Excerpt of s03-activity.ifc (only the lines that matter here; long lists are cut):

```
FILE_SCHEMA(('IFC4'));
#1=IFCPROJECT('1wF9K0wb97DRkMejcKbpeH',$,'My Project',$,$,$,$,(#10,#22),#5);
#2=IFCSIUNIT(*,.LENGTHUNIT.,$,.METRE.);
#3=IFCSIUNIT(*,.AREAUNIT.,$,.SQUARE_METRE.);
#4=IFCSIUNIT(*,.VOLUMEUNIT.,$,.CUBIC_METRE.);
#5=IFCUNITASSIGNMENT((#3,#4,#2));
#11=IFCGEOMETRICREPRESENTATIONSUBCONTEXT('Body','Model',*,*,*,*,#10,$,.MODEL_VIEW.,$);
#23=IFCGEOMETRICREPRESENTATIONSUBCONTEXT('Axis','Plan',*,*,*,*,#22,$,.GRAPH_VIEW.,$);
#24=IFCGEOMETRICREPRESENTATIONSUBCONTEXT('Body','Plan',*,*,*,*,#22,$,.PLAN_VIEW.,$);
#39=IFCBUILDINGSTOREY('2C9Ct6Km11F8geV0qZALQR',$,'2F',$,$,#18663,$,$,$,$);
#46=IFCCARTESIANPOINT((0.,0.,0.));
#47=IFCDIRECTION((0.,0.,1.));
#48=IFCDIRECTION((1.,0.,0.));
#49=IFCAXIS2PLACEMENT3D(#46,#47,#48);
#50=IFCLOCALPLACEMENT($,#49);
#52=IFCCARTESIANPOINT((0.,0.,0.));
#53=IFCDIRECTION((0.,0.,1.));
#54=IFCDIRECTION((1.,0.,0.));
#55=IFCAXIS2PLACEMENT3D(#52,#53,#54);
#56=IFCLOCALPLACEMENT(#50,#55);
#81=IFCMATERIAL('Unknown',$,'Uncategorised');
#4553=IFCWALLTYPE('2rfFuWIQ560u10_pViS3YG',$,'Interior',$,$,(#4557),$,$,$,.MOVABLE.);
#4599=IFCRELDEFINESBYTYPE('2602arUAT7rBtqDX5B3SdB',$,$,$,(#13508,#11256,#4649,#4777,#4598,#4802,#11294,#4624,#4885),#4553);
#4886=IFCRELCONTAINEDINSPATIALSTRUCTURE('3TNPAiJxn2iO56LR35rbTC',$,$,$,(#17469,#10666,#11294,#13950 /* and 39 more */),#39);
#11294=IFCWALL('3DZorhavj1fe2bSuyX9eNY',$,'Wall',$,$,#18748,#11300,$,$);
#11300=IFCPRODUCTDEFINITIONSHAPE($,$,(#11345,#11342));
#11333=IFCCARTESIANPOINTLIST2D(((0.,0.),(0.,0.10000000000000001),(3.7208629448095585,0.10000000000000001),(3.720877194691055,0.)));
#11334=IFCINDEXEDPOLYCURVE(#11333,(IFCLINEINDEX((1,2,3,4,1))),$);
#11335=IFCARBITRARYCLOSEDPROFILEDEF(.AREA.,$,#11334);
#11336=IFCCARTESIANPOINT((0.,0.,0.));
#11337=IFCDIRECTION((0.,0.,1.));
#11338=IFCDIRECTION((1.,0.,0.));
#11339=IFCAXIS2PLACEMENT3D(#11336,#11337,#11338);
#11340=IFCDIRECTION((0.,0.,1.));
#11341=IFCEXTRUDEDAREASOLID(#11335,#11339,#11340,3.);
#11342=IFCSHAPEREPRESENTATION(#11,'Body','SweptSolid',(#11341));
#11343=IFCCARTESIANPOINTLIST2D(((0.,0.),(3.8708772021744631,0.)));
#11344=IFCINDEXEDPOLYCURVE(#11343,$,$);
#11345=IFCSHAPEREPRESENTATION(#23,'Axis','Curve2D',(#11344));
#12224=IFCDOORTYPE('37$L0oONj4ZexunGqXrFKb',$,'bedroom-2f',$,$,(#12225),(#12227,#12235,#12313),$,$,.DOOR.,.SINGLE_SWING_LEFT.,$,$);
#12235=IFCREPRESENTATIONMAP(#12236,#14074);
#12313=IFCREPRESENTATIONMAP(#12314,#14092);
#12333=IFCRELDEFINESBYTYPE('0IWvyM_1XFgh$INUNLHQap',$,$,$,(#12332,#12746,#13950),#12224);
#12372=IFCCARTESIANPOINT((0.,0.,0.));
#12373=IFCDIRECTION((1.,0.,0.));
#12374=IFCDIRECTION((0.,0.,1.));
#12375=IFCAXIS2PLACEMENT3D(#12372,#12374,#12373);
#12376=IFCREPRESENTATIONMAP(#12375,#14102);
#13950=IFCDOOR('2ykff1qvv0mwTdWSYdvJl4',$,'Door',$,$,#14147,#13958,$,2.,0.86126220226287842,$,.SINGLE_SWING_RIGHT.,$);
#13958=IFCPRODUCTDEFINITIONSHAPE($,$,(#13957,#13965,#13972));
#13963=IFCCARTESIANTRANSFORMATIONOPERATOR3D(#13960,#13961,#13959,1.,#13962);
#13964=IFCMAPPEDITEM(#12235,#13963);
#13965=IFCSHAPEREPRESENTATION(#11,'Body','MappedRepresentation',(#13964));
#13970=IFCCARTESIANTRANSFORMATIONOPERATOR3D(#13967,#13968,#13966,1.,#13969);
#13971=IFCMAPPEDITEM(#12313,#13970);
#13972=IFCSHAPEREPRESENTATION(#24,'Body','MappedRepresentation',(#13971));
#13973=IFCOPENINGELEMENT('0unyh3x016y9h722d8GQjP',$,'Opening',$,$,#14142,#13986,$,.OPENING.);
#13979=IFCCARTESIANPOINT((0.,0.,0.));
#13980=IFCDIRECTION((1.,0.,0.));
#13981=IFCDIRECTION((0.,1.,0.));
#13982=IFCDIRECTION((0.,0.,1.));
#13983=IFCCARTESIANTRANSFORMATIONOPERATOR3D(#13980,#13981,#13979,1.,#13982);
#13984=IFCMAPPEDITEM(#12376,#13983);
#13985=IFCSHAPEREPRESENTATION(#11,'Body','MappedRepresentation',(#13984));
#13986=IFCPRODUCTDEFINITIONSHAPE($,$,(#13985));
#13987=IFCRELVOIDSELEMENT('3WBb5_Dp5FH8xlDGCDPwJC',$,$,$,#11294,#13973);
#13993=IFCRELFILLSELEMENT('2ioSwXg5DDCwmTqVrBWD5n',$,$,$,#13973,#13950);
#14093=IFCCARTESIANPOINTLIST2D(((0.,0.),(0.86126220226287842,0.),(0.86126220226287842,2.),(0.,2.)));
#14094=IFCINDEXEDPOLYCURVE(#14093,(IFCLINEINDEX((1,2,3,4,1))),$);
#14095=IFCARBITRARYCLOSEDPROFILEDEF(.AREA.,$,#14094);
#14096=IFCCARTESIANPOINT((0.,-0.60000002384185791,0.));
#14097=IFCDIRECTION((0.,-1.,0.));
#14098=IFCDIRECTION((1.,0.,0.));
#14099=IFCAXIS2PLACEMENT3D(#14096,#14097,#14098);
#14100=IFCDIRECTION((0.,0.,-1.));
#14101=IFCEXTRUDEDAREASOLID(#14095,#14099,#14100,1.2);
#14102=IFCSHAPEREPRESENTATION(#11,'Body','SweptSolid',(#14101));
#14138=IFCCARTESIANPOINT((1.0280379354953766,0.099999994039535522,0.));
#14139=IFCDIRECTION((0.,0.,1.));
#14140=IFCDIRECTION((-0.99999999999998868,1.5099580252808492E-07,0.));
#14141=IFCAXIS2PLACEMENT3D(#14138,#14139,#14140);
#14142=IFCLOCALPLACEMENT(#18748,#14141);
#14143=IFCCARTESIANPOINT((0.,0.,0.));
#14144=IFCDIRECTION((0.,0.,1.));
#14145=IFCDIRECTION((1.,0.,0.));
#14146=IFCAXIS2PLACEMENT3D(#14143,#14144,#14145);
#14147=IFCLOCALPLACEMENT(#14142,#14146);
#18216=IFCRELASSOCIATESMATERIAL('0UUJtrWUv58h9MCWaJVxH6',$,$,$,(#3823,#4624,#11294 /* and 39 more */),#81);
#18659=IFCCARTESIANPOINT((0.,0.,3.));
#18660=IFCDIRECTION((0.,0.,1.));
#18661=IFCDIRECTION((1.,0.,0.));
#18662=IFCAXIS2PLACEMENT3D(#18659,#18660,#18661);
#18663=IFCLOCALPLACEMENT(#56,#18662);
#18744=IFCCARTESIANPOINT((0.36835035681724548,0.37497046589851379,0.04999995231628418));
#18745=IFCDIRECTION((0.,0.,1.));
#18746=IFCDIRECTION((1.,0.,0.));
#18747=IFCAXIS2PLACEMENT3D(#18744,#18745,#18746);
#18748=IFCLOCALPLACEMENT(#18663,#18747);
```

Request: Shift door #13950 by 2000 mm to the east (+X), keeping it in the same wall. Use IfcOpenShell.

```python
import ifcopenshell
import ifcopenshell.api.geometry
import ifcopenshell.util.placement
import ifcopenshell.util.unit

model = ifcopenshell.open("s03-activity.ifc")
unit_scale = ifcopenshell.util.unit.calculate_unit_scale(model)

door = model.by_id(13950)
opening = door.FillsVoids[0].RelatingOpeningElement
wall = opening.VoidsElements[0].RelatingBuildingElement

wall_matrix = ifcopenshell.util.placement.get_local_placement(wall.ObjectPlacement)
shift = wall_matrix[:3, 0] * 2 / unit_scale
before = ifcopenshell.util.placement.get_local_placement(door.ObjectPlacement)[:3, 3].copy()

# The door is placed relative to its opening, so it follows when the opening moves.
matrix = ifcopenshell.util.placement.get_local_placement(opening.ObjectPlacement)
matrix[:3, 3] += shift
ifcopenshell.api.geometry.edit_object_placement(
    model, product=opening, matrix=matrix, is_si=False, should_transform_children=True
)

after = ifcopenshell.util.placement.get_local_placement(door.ObjectPlacement)[:3, 3]
print("door moved by", (after - before).round(3) + 0.0)

model.write("s03-activity_v2.ifc")
```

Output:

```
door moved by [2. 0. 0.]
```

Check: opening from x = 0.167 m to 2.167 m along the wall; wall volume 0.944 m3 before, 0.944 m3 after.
